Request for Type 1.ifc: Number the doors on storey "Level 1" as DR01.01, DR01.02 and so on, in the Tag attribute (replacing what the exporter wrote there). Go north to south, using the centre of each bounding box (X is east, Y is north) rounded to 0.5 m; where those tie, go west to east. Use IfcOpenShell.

First a look at what the model holds.

```python
import ifcopenshell
import ifcopenshell.util.element
import ifcopenshell.util.placement

model = ifcopenshell.open("Type 1.ifc")
print(model.schema)
storey = next(s for s in model.by_type("IfcBuildingStorey") if s.Name == "Level 1")
doors = [e for e in ifcopenshell.util.element.get_decomposition(storey) if e.is_a("IfcDoor")]
for e in sorted(doors, key=lambda e: e.id()):
    origin = ifcopenshell.util.placement.get_local_placement(e.ObjectPlacement)[:3, 3]
    print(e.id(), e.Tag, e.Name, origin.round(2) + 0.0, sep=" | ")
```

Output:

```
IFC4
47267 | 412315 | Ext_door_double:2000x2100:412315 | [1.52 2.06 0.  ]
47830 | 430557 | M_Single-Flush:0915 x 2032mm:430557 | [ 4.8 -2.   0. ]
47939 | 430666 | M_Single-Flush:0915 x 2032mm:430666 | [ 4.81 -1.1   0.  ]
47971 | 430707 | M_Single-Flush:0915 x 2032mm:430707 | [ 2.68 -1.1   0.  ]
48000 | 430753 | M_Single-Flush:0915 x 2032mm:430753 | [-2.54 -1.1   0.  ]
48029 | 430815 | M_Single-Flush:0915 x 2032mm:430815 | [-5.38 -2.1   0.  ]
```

```python
import ifcopenshell
import ifcopenshell.geom
import ifcopenshell.util.element
import ifcopenshell.util.shape

model = ifcopenshell.open("Type 1.ifc")
settings = ifcopenshell.geom.settings()
settings.set("use-world-coords", True)


def centre(element):
    shape = ifcopenshell.geom.create_shape(settings, element)
    return ifcopenshell.util.shape.get_bbox_centroid(shape.geometry)


storey = next(s for s in model.by_type("IfcBuildingStorey") if s.Name == "Level 1")
doors = [e for e in ifcopenshell.util.element.get_decomposition(storey) if e.is_a("IfcDoor")]

# Insertion points can sit at a corner or the storey origin, so sort by the geometry (in metres).
centres = {e: centre(e) for e in doors}
doors.sort(key=lambda e: (-round(centres[e][1] / 0.5), centres[e][0]))

for i, e in enumerate(doors, start=1):
    number = f"DR01.{i:02d}"
    e.Tag = number
    print(e.id(), number)

model.write("Type 1_updated.ifc")
```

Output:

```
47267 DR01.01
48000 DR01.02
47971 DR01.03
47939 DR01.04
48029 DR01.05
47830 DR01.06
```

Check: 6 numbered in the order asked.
